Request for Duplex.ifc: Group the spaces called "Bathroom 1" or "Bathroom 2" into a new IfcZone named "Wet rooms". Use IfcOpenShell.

First a look at what the model holds.

```python
import ifcopenshell

model = ifcopenshell.open("Duplex.ifc")
print(model.schema)
seen = {}
for space in model.by_type("IfcSpace"):
    seen[space.LongName] = seen.get(space.LongName, 0) + 1
for name, count in sorted(seen.items(), key=str):
    print(count, "x", name)
print("zones:", [z.Name for z in model.by_type("IfcZone")][:20])
```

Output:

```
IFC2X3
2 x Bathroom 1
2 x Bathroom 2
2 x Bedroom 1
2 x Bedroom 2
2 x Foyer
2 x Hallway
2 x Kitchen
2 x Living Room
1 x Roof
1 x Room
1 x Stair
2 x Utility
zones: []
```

```python
import ifcopenshell
import ifcopenshell.api.group
import ifcopenshell.api.root

model = ifcopenshell.open("Duplex.ifc")

names = {"Bathroom 1", "Bathroom 2"}
spaces = [s for s in model.by_type("IfcSpace") if s.LongName in names]

zone = ifcopenshell.api.root.create_entity(model, ifc_class="IfcZone", name="Wet rooms")
ifcopenshell.api.group.assign_group(model, products=spaces, group=zone)
print(len(spaces), "spaces in", zone.Name)

model.write("Duplex-out.ifc")
```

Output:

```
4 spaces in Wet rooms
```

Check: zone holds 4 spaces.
